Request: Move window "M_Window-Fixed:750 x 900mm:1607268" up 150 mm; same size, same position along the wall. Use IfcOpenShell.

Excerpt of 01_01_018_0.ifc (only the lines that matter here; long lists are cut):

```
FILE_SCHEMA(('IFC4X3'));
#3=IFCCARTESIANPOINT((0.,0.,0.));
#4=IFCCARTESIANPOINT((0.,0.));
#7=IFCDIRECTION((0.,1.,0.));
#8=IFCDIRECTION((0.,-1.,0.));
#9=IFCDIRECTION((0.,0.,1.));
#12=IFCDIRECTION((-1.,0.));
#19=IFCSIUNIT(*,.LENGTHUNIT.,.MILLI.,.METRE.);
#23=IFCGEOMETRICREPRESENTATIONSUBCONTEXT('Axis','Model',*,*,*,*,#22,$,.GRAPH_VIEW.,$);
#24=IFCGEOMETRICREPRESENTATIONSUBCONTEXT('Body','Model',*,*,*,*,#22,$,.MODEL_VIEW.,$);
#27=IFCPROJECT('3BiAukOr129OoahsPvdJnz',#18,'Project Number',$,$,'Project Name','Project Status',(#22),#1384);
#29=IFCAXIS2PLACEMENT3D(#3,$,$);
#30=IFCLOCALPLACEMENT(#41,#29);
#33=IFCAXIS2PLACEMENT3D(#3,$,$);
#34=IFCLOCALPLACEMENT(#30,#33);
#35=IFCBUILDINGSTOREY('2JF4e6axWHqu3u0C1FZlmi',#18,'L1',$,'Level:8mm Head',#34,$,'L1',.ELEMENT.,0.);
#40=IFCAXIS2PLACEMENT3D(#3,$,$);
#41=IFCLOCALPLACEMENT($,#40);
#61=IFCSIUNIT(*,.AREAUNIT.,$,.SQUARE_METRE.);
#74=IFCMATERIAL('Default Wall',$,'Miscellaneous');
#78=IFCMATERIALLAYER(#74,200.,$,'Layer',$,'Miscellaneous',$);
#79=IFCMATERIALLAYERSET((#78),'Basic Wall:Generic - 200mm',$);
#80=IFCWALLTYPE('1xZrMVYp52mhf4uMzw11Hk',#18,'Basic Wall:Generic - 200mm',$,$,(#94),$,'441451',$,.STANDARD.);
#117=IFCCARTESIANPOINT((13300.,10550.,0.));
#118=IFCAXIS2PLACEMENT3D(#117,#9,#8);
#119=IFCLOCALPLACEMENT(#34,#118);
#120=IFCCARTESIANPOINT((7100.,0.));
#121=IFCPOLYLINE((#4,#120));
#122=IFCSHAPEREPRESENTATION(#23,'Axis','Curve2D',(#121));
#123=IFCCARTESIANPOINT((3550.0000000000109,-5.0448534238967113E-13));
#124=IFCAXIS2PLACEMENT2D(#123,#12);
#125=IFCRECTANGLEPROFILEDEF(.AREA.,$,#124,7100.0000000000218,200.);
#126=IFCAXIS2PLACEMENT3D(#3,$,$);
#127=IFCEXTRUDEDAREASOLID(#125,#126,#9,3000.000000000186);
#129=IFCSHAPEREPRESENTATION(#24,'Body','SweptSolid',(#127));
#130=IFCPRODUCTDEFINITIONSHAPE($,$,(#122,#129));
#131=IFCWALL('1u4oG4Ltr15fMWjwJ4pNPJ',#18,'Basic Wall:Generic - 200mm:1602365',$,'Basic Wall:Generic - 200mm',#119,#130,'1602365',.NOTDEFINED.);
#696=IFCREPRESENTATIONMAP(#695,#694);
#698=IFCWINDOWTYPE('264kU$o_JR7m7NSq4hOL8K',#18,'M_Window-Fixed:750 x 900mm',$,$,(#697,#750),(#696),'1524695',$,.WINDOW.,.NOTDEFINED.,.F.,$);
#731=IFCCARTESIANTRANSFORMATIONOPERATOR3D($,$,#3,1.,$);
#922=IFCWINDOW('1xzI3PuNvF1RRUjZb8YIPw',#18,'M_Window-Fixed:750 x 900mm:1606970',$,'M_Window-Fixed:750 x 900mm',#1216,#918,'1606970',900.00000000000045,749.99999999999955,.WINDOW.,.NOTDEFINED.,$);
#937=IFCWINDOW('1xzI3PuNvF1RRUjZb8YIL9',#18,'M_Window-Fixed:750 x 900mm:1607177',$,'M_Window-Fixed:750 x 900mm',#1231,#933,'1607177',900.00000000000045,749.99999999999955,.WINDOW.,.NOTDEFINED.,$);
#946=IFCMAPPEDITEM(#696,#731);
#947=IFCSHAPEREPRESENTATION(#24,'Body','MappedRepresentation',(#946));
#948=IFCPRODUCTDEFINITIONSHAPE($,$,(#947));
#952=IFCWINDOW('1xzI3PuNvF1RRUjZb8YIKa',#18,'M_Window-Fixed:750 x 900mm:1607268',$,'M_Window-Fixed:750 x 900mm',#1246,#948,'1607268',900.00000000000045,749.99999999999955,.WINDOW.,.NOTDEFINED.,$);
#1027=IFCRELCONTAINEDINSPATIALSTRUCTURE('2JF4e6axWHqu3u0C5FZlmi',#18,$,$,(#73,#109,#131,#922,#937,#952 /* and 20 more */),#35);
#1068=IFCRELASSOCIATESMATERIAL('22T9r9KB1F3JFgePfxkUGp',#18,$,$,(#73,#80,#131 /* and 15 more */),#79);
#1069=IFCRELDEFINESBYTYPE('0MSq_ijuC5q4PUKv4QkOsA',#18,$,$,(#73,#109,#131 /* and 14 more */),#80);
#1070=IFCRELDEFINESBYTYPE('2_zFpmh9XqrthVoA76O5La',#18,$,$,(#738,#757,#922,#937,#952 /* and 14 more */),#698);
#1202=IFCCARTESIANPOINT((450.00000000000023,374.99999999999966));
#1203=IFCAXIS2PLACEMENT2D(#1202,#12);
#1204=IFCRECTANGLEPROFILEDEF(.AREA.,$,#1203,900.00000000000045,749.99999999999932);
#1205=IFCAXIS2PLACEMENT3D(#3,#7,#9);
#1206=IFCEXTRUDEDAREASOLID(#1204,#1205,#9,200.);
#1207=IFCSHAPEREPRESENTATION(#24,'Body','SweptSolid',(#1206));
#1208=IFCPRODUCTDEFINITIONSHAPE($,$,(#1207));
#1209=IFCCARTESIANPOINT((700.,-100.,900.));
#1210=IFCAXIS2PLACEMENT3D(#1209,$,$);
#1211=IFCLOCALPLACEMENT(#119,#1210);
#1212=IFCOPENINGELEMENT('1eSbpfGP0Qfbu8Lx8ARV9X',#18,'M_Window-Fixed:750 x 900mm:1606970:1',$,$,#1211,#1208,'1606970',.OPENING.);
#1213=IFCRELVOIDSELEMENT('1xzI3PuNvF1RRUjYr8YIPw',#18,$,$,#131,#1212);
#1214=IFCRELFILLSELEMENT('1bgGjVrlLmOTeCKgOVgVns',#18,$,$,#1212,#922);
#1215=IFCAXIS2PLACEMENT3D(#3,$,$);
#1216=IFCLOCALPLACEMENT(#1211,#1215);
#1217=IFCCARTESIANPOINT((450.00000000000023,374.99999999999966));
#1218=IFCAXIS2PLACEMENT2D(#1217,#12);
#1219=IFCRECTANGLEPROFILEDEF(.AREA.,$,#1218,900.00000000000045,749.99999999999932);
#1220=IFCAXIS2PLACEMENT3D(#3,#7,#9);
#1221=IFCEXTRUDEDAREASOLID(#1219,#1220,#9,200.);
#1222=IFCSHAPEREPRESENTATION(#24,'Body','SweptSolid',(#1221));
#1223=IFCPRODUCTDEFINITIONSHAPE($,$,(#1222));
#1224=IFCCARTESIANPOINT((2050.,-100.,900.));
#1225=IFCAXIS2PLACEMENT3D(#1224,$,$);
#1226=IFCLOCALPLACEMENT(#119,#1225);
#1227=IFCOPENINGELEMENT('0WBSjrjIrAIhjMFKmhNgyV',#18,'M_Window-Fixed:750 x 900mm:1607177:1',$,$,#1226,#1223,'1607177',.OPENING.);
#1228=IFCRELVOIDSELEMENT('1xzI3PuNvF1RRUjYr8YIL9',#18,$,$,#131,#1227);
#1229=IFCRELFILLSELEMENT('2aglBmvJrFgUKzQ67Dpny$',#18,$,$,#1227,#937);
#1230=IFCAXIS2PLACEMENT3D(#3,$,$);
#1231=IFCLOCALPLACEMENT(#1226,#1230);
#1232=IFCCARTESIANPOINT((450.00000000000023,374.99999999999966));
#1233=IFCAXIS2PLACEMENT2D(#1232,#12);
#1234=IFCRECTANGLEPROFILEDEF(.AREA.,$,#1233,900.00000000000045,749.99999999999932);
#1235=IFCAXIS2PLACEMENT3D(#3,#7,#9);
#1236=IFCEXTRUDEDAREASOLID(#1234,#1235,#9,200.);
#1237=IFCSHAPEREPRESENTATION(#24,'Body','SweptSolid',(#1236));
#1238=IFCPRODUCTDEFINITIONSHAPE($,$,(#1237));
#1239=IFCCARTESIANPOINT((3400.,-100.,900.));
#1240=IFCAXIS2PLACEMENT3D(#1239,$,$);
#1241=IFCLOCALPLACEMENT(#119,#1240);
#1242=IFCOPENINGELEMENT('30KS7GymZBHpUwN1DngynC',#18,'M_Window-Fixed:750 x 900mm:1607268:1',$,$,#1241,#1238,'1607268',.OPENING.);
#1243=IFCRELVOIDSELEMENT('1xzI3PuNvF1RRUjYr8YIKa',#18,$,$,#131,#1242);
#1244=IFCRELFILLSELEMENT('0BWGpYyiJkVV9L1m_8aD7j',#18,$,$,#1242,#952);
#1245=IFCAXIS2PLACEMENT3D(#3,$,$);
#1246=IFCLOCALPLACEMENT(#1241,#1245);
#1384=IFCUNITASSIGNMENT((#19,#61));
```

```python
import numpy as np
import ifcopenshell
import ifcopenshell.api.geometry
import ifcopenshell.util.placement
import ifcopenshell.util.unit

model = ifcopenshell.open("01_01_018_0.ifc")
unit_scale = ifcopenshell.util.unit.calculate_unit_scale(model)

window = model.by_guid("1xzI3PuNvF1RRUjZb8YIKa")
opening = window.FillsVoids[0].RelatingOpeningElement
dz = 150.0

shift = np.array([0.0, 0.0, dz])
# The window is placed relative to its opening, so it follows when the opening moves.
matrix = ifcopenshell.util.placement.get_local_placement(opening.ObjectPlacement)
matrix[:3, 3] += shift
ifcopenshell.api.geometry.edit_object_placement(
    model, product=opening, matrix=matrix, is_si=False, should_transform_children=True
)

print(f"moved by {dz * unit_scale:+.3f} m")

model.write("01_01_018_0_edited.ifc")
```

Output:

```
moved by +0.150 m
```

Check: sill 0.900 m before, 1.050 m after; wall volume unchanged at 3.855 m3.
